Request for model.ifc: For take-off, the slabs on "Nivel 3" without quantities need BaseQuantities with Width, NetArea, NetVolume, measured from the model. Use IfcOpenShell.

First a look at what the model holds.

```python
import ifcopenshell
import ifcopenshell.util.element
import ifcopenshell.util.unit

model = ifcopenshell.open("model.ifc")
print(model.schema)
for unit_type in ("LENGTHUNIT", "AREAUNIT", "VOLUMEUNIT"):
    print(unit_type, ifcopenshell.util.unit.calculate_unit_scale(model, unit_type))
storey = next(s for s in model.by_type("IfcBuildingStorey") if s.Name == "Nivel 3")
slabs = [e for e in ifcopenshell.util.element.get_decomposition(storey) if e.is_a("IfcSlab")]
for e in sorted(slabs, key=lambda e: e.id()):
    print(e.id(), e.is_a(), e.Name, list(ifcopenshell.util.element.get_psets(e, qtos_only=True)), sep=" | ")
```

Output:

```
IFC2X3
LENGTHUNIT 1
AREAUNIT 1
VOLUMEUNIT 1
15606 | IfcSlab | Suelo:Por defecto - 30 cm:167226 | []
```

```python
import ifcopenshell
import ifcopenshell.api.pset
import ifcopenshell.geom
import ifcopenshell.util.element
import ifcopenshell.util.shape
import ifcopenshell.util.unit

model = ifcopenshell.open("model.ifc")
unit_scale = ifcopenshell.util.unit.calculate_unit_scale(model)
area_scale = ifcopenshell.util.unit.calculate_unit_scale(model, "AREAUNIT")
volume_scale = ifcopenshell.util.unit.calculate_unit_scale(model, "VOLUMEUNIT")
settings = ifcopenshell.geom.settings()

storey = next(s for s in model.by_type("IfcBuildingStorey") if s.Name == "Nivel 3")
slabs = [e for e in ifcopenshell.util.element.get_decomposition(storey) if e.is_a("IfcSlab")]

for e in sorted(slabs, key=lambda e: e.id()):
    if ifcopenshell.util.element.get_psets(e, qtos_only=True, should_inherit=False):
        continue
    # Geometry comes back in metres, in the element's own axes.
    shape = ifcopenshell.geom.create_shape(settings, e)
    values = {
        "Width": ifcopenshell.util.shape.get_z(shape.geometry) / unit_scale,
        "NetArea": ifcopenshell.util.shape.get_footprint_area(shape.geometry) / area_scale,
        "NetVolume": ifcopenshell.util.shape.get_volume(shape.geometry) / volume_scale,
    }
    qto = ifcopenshell.api.pset.add_qto(model, product=e, name="BaseQuantities")
    ifcopenshell.api.pset.edit_qto(model, qto=qto, properties=values)
    print(e.id(), {k: round(v, 3) for k, v in values.items()})

model.write("model_rev.ifc")
```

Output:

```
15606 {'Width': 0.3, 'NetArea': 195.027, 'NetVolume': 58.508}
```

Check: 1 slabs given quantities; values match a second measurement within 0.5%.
